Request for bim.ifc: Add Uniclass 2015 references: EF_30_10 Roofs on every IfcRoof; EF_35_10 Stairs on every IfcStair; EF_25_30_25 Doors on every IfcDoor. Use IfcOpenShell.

First a look at what the model holds.

```python
import ifcopenshell

model = ifcopenshell.open("bim.ifc")
print(model.schema)
print("classifications:", [c.Name for c in model.by_type("IfcClassification")])
for ifc_class in ("IfcDoor", "IfcRoof", "IfcStair", "IfcWall", "IfcWindow"):
    print(ifc_class, len(model.by_type(ifc_class)))
```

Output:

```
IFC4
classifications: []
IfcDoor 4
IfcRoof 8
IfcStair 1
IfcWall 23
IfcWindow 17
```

```python
import ifcopenshell
import ifcopenshell.api.classification

model = ifcopenshell.open("bim.ifc")

system = ifcopenshell.api.classification.add_classification(model, classification="Uniclass 2015")

codes = {
    "IfcRoof": ("EF_30_10", "Roofs"),
    "IfcStair": ("EF_35_10", "Stairs"),
    "IfcDoor": ("EF_25_30_25", "Doors"),
}
for ifc_class, (code, name) in codes.items():
    products = model.by_type(ifc_class)
    ifcopenshell.api.classification.add_reference(
        model, products=products, classification=system, identification=code, name=name
    )
    print(code, len(products))

model.write("bim-out.ifc")
```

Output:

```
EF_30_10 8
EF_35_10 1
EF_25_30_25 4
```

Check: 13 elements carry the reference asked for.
